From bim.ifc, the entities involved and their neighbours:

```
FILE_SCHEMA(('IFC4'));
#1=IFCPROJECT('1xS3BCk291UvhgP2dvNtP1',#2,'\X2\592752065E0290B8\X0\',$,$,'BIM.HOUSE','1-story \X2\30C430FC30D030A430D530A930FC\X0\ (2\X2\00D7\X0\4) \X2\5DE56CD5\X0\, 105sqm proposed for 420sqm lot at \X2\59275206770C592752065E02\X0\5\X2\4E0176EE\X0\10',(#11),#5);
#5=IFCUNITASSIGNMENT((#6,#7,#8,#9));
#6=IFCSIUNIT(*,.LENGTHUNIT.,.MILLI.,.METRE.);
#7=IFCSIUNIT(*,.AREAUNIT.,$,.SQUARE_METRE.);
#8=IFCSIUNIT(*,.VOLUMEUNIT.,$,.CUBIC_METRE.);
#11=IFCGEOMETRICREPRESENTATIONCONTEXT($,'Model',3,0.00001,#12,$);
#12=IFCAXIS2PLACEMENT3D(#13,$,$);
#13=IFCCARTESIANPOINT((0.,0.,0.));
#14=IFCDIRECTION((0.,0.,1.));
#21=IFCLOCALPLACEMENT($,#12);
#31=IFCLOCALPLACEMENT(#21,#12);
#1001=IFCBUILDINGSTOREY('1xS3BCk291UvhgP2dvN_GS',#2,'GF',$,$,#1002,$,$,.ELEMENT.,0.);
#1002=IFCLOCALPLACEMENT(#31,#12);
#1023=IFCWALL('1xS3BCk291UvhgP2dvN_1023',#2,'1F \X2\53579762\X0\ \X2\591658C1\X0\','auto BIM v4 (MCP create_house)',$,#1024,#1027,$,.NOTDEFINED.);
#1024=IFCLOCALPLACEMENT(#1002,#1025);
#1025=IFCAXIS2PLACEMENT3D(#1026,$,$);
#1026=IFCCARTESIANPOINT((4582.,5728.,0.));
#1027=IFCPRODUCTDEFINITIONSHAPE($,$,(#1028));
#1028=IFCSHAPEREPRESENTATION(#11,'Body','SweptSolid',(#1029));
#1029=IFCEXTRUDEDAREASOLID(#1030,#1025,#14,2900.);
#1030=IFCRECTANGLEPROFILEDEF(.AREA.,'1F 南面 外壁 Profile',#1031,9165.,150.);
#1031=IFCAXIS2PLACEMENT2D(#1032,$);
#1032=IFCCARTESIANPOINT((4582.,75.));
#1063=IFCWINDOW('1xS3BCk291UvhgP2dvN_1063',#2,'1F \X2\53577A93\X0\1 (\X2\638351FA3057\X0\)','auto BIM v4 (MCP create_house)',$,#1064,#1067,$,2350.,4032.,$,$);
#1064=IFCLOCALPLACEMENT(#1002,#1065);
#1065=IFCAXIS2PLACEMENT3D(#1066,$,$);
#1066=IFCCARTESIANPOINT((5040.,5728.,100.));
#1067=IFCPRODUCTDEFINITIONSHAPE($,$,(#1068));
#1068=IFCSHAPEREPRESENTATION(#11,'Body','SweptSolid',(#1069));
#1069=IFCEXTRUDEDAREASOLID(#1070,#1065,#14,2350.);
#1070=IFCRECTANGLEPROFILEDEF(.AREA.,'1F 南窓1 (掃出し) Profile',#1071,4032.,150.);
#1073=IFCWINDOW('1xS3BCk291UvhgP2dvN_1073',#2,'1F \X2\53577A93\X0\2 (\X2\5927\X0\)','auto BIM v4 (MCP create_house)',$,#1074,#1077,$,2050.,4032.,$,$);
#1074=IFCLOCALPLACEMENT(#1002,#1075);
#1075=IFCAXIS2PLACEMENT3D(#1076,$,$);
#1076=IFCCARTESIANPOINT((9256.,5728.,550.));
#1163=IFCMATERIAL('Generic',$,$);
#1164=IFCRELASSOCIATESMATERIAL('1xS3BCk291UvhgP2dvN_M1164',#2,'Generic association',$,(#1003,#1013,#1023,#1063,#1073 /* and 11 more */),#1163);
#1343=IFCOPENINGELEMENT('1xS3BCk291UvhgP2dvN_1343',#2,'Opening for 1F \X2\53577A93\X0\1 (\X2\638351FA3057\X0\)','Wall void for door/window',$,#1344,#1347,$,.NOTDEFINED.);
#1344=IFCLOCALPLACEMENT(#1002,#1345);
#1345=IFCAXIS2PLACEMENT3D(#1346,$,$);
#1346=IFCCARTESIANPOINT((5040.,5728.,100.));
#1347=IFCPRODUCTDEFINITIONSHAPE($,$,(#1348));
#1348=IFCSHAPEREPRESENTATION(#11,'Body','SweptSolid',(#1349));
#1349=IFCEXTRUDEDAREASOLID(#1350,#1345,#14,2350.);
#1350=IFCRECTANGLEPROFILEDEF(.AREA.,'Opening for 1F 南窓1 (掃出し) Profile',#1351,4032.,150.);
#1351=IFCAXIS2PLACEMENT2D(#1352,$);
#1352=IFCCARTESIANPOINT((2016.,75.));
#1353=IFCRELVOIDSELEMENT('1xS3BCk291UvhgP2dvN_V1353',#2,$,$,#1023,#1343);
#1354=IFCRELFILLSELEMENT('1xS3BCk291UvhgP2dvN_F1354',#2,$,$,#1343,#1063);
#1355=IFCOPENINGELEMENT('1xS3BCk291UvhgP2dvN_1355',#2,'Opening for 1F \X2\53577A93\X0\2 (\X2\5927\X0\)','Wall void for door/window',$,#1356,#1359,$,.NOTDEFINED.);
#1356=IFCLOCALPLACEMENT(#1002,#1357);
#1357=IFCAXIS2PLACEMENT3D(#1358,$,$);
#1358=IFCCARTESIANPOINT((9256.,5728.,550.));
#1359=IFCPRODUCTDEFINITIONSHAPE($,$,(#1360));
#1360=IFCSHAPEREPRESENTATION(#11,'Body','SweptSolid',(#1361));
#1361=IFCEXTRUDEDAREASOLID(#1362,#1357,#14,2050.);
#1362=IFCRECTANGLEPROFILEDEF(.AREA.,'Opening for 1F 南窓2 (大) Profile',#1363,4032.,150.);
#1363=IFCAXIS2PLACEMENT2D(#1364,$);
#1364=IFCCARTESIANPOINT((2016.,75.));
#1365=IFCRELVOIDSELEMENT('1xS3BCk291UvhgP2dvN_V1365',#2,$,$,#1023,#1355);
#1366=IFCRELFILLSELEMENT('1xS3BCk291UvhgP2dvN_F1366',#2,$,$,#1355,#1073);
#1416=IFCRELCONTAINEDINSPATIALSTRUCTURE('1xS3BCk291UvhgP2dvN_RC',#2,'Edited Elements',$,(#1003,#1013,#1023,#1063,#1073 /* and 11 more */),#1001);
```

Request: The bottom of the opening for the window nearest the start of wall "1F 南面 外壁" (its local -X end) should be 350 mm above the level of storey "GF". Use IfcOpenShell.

```python
import numpy as np
import ifcopenshell
import ifcopenshell.api.geometry
import ifcopenshell.geom
import ifcopenshell.util.element
import ifcopenshell.util.placement
import ifcopenshell.util.shape
import ifcopenshell.util.unit

model = ifcopenshell.open("bim.ifc")
unit_scale = ifcopenshell.util.unit.calculate_unit_scale(model)

window = model.by_guid("1xS3BCk291UvhgP2dvN_1063")
opening = window.FillsVoids[0].RelatingOpeningElement
storey = ifcopenshell.util.element.get_container(window, ifc_class="IfcBuildingStorey")
level = ifcopenshell.util.placement.get_local_placement(storey.ObjectPlacement)[2, 3]

# The opening's origin need not be at the sill, so measure its lowest point.
shape = ifcopenshell.geom.create_shape(ifcopenshell.geom.settings(), opening)
bottom = ifcopenshell.util.shape.get_shape_bottom_elevation(shape, shape.geometry) / unit_scale
dz = level + 0.35 / unit_scale - bottom

shift = np.array([0.0, 0.0, dz])
# The window is not placed relative to its opening, so move both.
for product in (opening, window):
    matrix = ifcopenshell.util.placement.get_local_placement(product.ObjectPlacement)
    matrix[:3, 3] += shift
    ifcopenshell.api.geometry.edit_object_placement(model, product=product, matrix=matrix, is_si=False)

print(f"moved by {dz * unit_scale:+.3f} m")

model.write("bim_v2.ifc")
```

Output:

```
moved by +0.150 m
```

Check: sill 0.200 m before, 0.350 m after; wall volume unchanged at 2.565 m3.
